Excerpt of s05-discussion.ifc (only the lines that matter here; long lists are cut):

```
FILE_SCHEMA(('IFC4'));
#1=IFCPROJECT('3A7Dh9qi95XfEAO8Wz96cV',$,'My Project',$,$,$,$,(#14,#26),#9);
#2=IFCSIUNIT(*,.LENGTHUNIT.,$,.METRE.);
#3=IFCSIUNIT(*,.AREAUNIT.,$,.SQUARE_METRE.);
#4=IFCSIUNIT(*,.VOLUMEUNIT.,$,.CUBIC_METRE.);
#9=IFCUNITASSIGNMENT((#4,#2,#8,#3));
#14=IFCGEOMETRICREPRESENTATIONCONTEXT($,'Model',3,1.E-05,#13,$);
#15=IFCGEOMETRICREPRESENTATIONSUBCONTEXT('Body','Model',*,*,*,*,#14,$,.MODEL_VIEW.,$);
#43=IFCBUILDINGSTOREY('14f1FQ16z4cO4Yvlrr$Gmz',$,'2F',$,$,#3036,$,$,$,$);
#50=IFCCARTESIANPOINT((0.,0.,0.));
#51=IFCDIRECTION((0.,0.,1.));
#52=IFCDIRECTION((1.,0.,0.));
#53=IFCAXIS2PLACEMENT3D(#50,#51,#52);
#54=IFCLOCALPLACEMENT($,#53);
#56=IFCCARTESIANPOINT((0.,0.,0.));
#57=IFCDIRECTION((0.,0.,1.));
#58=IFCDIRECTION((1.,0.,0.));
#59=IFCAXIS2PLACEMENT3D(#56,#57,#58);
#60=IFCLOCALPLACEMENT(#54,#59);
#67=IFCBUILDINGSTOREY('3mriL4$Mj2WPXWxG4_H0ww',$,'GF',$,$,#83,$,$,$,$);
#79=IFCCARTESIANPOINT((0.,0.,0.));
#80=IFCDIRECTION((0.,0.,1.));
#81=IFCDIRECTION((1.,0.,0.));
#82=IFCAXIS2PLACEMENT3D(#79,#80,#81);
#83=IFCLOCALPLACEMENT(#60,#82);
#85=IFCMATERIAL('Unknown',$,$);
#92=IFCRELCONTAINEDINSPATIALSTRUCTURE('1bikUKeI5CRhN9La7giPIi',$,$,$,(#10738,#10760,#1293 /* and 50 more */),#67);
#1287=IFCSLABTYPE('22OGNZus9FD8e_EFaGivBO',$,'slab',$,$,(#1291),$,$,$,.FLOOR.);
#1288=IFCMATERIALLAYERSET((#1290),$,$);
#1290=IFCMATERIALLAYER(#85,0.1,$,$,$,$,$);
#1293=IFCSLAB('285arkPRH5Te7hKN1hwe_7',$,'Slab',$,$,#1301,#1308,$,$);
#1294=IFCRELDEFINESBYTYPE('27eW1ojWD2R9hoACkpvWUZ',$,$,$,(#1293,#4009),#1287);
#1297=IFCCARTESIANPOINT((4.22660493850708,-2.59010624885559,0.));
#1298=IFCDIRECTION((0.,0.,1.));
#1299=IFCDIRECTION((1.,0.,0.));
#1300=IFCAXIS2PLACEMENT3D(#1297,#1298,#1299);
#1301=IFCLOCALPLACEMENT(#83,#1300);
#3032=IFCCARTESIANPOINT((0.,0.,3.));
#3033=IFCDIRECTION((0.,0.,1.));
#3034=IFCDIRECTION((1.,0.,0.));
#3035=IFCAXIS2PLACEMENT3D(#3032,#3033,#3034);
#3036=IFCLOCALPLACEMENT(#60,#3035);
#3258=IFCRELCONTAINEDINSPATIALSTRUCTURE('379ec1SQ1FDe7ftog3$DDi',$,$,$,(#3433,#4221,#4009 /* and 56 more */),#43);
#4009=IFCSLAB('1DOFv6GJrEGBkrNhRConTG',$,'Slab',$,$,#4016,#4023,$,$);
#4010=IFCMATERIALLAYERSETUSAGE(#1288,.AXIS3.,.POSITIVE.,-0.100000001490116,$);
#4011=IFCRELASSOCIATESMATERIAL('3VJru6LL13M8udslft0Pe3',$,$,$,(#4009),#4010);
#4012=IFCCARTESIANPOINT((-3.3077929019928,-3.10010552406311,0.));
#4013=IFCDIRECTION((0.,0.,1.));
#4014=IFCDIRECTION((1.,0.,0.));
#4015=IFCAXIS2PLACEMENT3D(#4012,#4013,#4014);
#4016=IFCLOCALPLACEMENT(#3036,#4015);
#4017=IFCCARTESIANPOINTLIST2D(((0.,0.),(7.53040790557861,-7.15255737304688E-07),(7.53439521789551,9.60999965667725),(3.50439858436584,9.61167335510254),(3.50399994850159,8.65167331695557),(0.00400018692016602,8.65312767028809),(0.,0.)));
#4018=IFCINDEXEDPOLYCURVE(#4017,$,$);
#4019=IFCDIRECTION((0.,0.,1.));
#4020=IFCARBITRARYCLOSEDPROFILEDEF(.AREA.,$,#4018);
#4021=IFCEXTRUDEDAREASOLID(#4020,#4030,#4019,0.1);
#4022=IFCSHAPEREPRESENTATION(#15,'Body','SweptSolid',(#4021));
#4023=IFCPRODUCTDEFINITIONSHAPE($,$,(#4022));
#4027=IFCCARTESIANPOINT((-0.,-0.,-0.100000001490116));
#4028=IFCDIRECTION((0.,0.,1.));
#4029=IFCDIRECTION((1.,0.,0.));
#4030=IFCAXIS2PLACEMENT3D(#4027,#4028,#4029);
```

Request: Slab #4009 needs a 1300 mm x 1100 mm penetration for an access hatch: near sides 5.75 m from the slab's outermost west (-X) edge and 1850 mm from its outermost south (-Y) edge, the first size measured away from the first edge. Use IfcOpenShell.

```python
import numpy as np
import ifcopenshell
import ifcopenshell.api.feature
import ifcopenshell.api.geometry
import ifcopenshell.api.root
import ifcopenshell.geom
import ifcopenshell.util.placement
import ifcopenshell.util.representation
import ifcopenshell.util.shape
import ifcopenshell.util.unit

model = ifcopenshell.open("s05-discussion.ifc")
unit_scale = ifcopenshell.util.unit.calculate_unit_scale(model)
settings = ifcopenshell.geom.settings()


def volume(element):
    """Net volume in cubic metres, openings subtracted."""
    shape = ifcopenshell.geom.create_shape(settings, element)
    return ifcopenshell.util.shape.get_volume(shape.geometry)


slab = model.by_guid("1DOFv6GJrEGBkrNhRConTG")
before = volume(slab)

# Extent in the slab's own axes, in metres. The edges named are its -X and -Y sides.
slab_shape = ifcopenshell.geom.create_shape(settings, slab)
vertices = ifcopenshell.util.shape.get_vertices(slab_shape.geometry)
x_min, y_min, bottom = vertices.min(axis=0)
top = vertices[:, 2].max()

opening = ifcopenshell.api.root.create_entity(model, ifc_class="IfcOpeningElement", name="Access hatch opening", predefined_type="OPENING")
context = ifcopenshell.util.representation.get_context(model, "Model", "Body", "MODEL_VIEW")
width, depth = 1.3, 1.1
outline = [(0.0, 0.0), (width, 0.0), (width, depth), (0.0, depth), (0.0, 0.0)]
# Overshoot both faces by 50 mm so the cut is clean.
shape = ifcopenshell.api.geometry.add_slab_representation(
    model, context=context, depth=top - bottom + 0.1, polyline=outline
)
ifcopenshell.api.geometry.assign_representation(model, product=opening, representation=shape)

matrix = ifcopenshell.util.placement.get_local_placement(slab.ObjectPlacement)
matrix[:, 3] = matrix @ np.append(np.array([x_min + 5.75, y_min + 1.85, bottom - 0.05]) / unit_scale, 1.0)
ifcopenshell.api.geometry.edit_object_placement(model, product=opening, matrix=matrix, is_si=False)
ifcopenshell.api.feature.add_feature(model, feature=opening, element=slab)

after = volume(slab)

print(f"slab volume {before:.3f} -> {after:.3f} m3")

model.write("s05-discussion_updated.ifc")
```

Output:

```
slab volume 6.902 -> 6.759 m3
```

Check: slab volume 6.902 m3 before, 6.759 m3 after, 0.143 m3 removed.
